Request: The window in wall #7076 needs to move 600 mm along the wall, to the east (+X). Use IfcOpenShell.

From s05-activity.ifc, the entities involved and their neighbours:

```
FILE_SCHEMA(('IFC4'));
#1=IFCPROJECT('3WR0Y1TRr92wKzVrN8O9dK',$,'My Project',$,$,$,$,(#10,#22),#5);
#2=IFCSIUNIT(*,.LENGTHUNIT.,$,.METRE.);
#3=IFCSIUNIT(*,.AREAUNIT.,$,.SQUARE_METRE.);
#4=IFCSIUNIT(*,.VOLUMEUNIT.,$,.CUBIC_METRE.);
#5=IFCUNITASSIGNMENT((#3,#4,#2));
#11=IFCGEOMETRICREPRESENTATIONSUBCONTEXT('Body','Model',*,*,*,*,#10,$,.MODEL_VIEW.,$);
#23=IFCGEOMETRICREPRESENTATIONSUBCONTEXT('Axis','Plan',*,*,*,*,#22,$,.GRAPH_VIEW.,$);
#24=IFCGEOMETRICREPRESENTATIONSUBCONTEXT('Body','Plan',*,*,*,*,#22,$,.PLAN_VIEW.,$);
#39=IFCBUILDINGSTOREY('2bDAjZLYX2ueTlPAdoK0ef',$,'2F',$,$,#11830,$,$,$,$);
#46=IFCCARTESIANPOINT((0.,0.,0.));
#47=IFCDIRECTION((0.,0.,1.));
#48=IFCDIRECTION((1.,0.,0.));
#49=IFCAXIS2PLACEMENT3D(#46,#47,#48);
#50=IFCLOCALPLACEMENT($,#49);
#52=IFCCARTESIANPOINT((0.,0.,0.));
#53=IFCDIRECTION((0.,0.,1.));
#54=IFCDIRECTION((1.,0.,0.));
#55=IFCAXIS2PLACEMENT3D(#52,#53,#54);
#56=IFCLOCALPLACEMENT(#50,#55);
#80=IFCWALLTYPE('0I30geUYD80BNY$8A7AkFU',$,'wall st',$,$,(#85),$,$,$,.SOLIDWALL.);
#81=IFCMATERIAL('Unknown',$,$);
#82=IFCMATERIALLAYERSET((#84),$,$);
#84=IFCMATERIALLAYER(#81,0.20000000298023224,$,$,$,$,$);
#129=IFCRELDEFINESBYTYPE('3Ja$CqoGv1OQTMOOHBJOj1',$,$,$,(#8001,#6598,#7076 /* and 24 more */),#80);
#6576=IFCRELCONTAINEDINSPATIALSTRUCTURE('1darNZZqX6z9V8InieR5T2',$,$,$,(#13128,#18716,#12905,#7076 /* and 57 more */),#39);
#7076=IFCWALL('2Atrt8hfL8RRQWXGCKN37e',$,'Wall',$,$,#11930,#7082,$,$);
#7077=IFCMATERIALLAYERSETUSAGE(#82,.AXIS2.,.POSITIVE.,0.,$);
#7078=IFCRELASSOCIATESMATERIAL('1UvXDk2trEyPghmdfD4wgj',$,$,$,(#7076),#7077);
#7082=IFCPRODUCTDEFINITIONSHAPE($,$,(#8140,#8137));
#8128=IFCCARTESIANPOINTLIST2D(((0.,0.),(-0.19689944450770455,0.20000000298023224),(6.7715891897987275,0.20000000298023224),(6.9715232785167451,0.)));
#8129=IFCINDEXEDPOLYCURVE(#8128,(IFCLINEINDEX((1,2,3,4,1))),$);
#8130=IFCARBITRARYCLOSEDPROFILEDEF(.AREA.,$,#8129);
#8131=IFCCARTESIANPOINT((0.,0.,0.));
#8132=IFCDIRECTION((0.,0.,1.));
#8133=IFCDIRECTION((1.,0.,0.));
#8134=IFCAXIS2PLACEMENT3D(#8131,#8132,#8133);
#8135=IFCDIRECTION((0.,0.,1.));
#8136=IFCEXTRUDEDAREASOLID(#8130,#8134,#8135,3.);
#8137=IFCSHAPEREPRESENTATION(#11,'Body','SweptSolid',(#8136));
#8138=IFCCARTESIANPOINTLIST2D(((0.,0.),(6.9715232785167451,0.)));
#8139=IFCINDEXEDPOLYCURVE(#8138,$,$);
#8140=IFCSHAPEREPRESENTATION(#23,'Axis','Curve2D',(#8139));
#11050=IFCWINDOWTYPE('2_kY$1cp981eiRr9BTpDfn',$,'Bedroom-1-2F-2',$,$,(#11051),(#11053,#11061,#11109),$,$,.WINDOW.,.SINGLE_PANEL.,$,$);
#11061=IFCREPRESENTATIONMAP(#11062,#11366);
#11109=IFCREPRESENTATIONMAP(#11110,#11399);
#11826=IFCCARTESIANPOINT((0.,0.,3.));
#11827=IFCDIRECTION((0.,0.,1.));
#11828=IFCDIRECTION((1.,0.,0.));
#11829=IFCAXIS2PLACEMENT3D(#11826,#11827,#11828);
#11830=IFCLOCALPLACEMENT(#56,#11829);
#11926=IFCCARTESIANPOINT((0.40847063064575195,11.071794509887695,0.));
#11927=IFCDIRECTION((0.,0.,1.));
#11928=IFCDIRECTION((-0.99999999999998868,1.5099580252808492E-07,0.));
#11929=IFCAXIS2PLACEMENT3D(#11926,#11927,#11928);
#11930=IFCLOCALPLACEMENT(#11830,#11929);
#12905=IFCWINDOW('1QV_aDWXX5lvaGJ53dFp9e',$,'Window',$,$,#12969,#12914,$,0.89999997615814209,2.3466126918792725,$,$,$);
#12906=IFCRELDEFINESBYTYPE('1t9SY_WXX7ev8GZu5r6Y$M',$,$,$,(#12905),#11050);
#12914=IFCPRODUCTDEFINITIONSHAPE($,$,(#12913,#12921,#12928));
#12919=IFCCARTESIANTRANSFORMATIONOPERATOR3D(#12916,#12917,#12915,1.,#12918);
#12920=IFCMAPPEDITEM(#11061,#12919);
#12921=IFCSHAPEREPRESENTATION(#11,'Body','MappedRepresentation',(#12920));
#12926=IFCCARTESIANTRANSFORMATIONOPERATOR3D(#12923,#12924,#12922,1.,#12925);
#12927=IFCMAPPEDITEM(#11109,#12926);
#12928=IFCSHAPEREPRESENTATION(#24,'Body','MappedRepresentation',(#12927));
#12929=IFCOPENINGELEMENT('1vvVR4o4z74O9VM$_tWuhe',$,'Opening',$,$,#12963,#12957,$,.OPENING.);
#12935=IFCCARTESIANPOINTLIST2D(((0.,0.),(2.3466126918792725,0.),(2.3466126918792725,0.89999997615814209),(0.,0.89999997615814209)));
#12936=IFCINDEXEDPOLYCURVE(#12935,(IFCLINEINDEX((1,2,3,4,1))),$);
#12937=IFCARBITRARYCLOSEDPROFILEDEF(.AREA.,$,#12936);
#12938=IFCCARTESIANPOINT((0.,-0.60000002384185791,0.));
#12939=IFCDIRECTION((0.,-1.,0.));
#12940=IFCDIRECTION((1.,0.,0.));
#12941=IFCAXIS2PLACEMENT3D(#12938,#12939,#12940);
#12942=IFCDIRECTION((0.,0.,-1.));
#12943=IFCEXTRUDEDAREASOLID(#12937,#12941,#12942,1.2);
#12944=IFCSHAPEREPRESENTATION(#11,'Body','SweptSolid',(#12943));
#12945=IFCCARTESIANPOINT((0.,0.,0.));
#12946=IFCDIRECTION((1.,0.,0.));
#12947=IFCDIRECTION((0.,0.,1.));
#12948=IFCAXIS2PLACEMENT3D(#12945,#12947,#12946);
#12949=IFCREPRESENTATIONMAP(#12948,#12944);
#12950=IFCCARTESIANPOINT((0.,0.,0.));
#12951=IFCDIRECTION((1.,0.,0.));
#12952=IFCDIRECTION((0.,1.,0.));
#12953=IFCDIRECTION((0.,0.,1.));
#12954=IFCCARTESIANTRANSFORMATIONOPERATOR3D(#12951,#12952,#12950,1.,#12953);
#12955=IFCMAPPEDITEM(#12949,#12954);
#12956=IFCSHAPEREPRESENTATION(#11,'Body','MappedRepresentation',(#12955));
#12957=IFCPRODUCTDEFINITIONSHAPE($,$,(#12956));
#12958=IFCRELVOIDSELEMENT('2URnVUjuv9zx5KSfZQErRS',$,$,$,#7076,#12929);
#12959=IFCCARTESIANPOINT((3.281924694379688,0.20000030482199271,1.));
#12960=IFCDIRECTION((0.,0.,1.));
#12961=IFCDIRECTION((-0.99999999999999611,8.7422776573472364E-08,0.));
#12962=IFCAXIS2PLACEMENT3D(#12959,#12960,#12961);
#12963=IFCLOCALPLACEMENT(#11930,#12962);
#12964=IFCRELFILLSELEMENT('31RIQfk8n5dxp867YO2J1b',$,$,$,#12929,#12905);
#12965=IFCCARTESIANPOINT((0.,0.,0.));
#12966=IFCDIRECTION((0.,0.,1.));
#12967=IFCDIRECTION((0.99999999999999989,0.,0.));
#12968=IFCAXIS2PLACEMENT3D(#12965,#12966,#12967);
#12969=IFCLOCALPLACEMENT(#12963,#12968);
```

```python
import ifcopenshell
import ifcopenshell.api.geometry
import ifcopenshell.util.placement
import ifcopenshell.util.unit

model = ifcopenshell.open("s05-activity.ifc")
unit_scale = ifcopenshell.util.unit.calculate_unit_scale(model)

window = model.by_guid("1QV_aDWXX5lvaGJ53dFp9e")
opening = window.FillsVoids[0].RelatingOpeningElement
wall = opening.VoidsElements[0].RelatingBuildingElement

wall_matrix = ifcopenshell.util.placement.get_local_placement(wall.ObjectPlacement)
shift = wall_matrix[:3, 0] * -0.6 / unit_scale
before = ifcopenshell.util.placement.get_local_placement(window.ObjectPlacement)[:3, 3].copy()

# The window is placed relative to its opening, so it follows when the opening moves.
matrix = ifcopenshell.util.placement.get_local_placement(opening.ObjectPlacement)
matrix[:3, 3] += shift
ifcopenshell.api.geometry.edit_object_placement(
    model, product=opening, matrix=matrix, is_si=False, should_transform_children=True
)

after = ifcopenshell.util.placement.get_local_placement(window.ObjectPlacement)[:3, 3]
print("window moved by", (after - before).round(3) + 0.0)

model.write("s05-activity_rev.ifc")
```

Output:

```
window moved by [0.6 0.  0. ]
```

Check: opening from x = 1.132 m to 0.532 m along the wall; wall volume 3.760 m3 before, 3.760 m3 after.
